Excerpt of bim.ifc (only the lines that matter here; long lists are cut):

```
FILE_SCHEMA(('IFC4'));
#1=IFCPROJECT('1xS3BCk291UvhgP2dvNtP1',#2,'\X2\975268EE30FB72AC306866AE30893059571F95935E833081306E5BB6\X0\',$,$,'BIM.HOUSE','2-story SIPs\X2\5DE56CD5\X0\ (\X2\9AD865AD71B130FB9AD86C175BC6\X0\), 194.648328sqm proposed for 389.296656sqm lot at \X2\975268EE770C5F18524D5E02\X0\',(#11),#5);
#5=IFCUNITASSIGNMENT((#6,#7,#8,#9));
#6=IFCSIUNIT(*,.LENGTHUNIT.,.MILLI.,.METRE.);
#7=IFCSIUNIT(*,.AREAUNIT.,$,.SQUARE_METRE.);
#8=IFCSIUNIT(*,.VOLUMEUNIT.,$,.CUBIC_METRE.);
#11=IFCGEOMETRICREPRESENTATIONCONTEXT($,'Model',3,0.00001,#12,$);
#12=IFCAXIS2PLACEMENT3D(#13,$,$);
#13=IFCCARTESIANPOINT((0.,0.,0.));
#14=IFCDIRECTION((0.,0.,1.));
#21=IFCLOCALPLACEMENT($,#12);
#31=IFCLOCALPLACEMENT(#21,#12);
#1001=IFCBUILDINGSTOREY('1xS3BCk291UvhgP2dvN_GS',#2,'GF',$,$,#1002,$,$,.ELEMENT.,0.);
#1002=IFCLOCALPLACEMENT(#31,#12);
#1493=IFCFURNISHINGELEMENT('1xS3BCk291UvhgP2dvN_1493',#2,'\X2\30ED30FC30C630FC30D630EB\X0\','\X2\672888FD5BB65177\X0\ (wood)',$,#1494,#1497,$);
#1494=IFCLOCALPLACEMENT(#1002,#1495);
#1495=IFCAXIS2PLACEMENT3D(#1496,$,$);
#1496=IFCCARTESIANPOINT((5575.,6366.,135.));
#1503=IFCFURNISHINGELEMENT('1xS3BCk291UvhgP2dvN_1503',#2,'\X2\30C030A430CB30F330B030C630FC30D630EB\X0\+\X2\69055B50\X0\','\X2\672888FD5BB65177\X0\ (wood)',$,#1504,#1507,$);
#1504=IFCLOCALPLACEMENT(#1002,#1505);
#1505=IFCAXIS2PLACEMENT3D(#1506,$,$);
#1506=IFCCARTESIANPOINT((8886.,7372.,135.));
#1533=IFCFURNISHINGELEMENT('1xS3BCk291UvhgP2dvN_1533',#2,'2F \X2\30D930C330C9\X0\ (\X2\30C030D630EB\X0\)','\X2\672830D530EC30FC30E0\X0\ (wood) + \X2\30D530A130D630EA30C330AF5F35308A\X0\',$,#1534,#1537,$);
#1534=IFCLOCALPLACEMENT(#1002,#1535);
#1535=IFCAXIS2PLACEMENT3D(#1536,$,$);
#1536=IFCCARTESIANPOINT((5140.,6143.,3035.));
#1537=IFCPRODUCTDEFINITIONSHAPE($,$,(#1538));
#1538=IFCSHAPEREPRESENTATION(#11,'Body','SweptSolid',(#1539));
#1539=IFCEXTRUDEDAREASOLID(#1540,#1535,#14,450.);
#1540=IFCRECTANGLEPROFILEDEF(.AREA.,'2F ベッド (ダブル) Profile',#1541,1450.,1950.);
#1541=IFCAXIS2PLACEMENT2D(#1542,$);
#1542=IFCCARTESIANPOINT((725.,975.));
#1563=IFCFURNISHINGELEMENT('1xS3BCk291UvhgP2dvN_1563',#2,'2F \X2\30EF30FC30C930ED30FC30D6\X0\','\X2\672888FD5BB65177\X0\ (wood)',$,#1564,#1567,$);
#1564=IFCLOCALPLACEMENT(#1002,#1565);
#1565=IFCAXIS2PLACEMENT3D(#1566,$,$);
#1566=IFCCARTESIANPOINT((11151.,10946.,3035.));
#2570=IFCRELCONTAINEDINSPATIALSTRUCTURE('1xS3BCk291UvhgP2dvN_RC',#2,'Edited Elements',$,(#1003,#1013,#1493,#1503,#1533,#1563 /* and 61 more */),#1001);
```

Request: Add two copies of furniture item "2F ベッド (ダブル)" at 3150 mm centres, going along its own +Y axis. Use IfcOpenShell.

```python
import ifcopenshell
import ifcopenshell.api.geometry
import ifcopenshell.api.root
import ifcopenshell.util.element
import ifcopenshell.util.placement
import ifcopenshell.util.unit

model = ifcopenshell.open("bim.ifc")
unit_scale = ifcopenshell.util.unit.calculate_unit_scale(model)


def reuse_history(source, copy):
    """copy_class also copies each property set's owner history, people and application; keep the originals."""
    for rel in copy.IsDefinedBy:
        if rel.is_a("IfcRelDefinesByProperties") and (history := rel.RelatingPropertyDefinition.OwnerHistory):
            rel.RelatingPropertyDefinition.OwnerHistory = source.OwnerHistory
            ifcopenshell.util.element.remove_deep2(model, history)


source = model.by_guid("1xS3BCk291UvhgP2dvN_1533")
base = ifcopenshell.util.placement.get_local_placement(source.ObjectPlacement)
step = base[:3, 1] * 3.15 / unit_scale

for i in range(1, 3):
    copy = ifcopenshell.api.root.copy_class(model, product=source)
    copy.Representation = ifcopenshell.util.element.copy_deep(
        model, source.Representation, exclude=["IfcGeometricRepresentationContext", "IfcRepresentationMap"]
    )
    reuse_history(source, copy)
    matrix = base.copy()
    matrix[:3, 3] += i * step
    print("added at", matrix[:3, 3].round(3) + 0.0)
    ifcopenshell.api.geometry.edit_object_placement(model, product=copy, matrix=matrix, is_si=False)

model.write("bim-out.ifc")
```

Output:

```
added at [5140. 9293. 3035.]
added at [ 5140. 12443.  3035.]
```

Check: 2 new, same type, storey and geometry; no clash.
